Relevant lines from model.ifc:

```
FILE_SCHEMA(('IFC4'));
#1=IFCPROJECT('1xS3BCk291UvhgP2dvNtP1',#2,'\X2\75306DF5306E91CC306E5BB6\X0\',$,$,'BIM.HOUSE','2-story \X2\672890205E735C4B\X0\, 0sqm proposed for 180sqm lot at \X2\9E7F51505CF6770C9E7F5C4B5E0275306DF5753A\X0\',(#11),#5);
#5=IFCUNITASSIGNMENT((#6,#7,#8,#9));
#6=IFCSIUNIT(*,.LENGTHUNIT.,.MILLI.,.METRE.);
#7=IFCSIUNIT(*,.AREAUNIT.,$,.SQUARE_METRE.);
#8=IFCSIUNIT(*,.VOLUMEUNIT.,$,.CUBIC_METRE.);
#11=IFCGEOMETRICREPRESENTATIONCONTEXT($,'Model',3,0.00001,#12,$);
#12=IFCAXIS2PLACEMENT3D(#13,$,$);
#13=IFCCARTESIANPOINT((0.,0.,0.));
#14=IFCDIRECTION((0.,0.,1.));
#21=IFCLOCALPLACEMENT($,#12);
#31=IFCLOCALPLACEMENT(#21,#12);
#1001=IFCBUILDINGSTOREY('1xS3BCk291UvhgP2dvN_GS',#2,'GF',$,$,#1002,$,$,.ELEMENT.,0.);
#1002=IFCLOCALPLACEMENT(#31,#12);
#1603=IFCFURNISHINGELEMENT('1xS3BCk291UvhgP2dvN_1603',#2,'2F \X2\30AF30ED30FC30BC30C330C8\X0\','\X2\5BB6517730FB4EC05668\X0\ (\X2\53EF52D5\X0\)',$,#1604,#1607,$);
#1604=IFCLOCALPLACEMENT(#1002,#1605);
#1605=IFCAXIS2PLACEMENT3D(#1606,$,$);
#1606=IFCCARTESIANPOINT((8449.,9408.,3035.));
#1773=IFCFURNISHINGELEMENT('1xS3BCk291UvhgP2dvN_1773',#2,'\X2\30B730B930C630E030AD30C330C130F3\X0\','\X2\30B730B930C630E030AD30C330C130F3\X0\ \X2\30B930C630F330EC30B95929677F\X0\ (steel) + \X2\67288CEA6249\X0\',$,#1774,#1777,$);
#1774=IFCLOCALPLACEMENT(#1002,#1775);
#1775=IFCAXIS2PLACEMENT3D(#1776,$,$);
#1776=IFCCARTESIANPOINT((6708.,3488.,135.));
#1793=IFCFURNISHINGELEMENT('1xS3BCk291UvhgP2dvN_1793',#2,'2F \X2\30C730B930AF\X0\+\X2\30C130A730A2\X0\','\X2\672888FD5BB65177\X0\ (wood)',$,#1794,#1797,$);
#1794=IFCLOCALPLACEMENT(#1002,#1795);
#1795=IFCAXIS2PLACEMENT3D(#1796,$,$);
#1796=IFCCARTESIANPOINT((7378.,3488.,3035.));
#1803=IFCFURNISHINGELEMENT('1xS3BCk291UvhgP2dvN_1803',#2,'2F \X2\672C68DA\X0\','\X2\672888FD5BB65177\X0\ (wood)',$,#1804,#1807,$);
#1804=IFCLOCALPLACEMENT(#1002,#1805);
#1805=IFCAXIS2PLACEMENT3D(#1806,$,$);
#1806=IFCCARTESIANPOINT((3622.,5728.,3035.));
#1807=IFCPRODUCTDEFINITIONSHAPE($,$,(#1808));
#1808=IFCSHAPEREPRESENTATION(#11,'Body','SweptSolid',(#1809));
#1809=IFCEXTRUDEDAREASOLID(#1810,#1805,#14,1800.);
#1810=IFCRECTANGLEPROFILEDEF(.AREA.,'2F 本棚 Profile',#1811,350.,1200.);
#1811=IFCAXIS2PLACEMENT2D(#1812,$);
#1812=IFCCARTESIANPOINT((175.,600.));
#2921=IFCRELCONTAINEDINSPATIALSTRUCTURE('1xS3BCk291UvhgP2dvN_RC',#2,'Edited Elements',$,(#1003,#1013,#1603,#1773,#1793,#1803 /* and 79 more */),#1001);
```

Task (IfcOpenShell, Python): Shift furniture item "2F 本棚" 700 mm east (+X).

```python
import ifcopenshell
import ifcopenshell.api.geometry
import ifcopenshell.util.placement

model = ifcopenshell.open("model.ifc")

item = model.by_guid("1xS3BCk291UvhgP2dvN_1803")
matrix = ifcopenshell.util.placement.get_local_placement(item.ObjectPlacement)
matrix[0, 3] += 700.0
ifcopenshell.api.geometry.edit_object_placement(model, product=item, matrix=matrix, is_si=False)

print(ifcopenshell.util.placement.get_local_placement(item.ObjectPlacement).round(3) + 0.0)

model.write("model_rev.ifc")
```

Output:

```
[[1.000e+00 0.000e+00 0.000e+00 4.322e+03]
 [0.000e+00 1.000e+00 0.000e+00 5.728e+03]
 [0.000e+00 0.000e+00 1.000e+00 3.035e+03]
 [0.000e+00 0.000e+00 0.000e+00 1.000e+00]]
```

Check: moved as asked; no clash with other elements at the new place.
